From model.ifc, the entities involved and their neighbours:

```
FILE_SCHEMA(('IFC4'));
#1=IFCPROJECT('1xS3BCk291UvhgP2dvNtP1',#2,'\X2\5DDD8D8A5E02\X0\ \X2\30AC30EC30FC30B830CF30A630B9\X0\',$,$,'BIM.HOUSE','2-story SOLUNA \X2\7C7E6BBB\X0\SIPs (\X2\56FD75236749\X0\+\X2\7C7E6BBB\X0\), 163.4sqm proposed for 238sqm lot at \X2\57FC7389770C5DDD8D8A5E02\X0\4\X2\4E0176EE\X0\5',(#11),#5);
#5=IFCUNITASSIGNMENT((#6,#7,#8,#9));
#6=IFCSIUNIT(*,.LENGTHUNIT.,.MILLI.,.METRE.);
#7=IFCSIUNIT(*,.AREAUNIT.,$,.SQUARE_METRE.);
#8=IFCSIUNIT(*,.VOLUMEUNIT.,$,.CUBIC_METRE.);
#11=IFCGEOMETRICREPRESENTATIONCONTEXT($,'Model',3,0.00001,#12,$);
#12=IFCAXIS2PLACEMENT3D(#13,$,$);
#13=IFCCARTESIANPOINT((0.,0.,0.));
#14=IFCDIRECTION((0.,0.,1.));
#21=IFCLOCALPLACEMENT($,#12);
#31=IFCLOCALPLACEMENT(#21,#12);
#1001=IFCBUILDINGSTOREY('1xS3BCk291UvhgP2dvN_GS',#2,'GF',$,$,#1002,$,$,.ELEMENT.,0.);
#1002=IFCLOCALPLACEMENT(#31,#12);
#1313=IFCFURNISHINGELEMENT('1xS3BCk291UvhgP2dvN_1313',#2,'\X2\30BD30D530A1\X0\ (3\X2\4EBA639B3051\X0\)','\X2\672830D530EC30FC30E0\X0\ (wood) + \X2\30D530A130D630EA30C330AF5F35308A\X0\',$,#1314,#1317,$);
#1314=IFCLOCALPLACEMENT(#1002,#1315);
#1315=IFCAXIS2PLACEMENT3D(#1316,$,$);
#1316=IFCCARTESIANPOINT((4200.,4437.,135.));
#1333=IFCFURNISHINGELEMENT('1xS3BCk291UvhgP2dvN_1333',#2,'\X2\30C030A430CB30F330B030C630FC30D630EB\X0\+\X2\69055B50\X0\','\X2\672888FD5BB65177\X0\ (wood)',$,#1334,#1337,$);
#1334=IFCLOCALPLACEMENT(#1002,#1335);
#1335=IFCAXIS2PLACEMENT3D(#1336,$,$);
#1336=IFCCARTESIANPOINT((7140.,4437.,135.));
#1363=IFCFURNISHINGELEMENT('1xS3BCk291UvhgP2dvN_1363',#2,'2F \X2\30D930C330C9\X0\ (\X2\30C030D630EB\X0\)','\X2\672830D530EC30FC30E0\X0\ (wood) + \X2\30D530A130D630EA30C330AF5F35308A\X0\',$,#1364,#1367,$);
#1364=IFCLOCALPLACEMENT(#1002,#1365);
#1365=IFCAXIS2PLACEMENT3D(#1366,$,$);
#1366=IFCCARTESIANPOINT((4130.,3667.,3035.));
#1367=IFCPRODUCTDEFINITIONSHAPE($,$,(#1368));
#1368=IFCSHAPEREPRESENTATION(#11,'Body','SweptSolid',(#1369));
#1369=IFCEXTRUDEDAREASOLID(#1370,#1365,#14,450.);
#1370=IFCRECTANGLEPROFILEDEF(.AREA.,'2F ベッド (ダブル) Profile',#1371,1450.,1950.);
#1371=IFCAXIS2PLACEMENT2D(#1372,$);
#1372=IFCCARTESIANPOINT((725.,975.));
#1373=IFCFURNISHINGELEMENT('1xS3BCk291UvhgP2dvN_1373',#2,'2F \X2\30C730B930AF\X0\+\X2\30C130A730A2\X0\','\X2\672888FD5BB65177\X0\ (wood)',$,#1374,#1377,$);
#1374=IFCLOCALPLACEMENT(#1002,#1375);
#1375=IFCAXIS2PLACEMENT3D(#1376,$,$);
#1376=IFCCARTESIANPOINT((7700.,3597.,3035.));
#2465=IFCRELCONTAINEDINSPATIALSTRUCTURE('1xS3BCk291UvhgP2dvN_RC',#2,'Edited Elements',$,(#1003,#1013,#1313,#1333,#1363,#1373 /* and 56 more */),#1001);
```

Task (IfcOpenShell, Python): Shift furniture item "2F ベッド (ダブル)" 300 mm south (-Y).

```python
import ifcopenshell
import ifcopenshell.api.geometry
import ifcopenshell.util.placement
import ifcopenshell.util.unit

model = ifcopenshell.open("model.ifc")
unit_scale = ifcopenshell.util.unit.calculate_unit_scale(model)

item = model.by_guid("1xS3BCk291UvhgP2dvN_1363")
matrix = ifcopenshell.util.placement.get_local_placement(item.ObjectPlacement)
matrix[1, 3] -= 0.3 / unit_scale
ifcopenshell.api.geometry.edit_object_placement(model, product=item, matrix=matrix, is_si=False)

print(ifcopenshell.util.placement.get_local_placement(item.ObjectPlacement).round(3) + 0.0)

model.write("model_rev.ifc")
```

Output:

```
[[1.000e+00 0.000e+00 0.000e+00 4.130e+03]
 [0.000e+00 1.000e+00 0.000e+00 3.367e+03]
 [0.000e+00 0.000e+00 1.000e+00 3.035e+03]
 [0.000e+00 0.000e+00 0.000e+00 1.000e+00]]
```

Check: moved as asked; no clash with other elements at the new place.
